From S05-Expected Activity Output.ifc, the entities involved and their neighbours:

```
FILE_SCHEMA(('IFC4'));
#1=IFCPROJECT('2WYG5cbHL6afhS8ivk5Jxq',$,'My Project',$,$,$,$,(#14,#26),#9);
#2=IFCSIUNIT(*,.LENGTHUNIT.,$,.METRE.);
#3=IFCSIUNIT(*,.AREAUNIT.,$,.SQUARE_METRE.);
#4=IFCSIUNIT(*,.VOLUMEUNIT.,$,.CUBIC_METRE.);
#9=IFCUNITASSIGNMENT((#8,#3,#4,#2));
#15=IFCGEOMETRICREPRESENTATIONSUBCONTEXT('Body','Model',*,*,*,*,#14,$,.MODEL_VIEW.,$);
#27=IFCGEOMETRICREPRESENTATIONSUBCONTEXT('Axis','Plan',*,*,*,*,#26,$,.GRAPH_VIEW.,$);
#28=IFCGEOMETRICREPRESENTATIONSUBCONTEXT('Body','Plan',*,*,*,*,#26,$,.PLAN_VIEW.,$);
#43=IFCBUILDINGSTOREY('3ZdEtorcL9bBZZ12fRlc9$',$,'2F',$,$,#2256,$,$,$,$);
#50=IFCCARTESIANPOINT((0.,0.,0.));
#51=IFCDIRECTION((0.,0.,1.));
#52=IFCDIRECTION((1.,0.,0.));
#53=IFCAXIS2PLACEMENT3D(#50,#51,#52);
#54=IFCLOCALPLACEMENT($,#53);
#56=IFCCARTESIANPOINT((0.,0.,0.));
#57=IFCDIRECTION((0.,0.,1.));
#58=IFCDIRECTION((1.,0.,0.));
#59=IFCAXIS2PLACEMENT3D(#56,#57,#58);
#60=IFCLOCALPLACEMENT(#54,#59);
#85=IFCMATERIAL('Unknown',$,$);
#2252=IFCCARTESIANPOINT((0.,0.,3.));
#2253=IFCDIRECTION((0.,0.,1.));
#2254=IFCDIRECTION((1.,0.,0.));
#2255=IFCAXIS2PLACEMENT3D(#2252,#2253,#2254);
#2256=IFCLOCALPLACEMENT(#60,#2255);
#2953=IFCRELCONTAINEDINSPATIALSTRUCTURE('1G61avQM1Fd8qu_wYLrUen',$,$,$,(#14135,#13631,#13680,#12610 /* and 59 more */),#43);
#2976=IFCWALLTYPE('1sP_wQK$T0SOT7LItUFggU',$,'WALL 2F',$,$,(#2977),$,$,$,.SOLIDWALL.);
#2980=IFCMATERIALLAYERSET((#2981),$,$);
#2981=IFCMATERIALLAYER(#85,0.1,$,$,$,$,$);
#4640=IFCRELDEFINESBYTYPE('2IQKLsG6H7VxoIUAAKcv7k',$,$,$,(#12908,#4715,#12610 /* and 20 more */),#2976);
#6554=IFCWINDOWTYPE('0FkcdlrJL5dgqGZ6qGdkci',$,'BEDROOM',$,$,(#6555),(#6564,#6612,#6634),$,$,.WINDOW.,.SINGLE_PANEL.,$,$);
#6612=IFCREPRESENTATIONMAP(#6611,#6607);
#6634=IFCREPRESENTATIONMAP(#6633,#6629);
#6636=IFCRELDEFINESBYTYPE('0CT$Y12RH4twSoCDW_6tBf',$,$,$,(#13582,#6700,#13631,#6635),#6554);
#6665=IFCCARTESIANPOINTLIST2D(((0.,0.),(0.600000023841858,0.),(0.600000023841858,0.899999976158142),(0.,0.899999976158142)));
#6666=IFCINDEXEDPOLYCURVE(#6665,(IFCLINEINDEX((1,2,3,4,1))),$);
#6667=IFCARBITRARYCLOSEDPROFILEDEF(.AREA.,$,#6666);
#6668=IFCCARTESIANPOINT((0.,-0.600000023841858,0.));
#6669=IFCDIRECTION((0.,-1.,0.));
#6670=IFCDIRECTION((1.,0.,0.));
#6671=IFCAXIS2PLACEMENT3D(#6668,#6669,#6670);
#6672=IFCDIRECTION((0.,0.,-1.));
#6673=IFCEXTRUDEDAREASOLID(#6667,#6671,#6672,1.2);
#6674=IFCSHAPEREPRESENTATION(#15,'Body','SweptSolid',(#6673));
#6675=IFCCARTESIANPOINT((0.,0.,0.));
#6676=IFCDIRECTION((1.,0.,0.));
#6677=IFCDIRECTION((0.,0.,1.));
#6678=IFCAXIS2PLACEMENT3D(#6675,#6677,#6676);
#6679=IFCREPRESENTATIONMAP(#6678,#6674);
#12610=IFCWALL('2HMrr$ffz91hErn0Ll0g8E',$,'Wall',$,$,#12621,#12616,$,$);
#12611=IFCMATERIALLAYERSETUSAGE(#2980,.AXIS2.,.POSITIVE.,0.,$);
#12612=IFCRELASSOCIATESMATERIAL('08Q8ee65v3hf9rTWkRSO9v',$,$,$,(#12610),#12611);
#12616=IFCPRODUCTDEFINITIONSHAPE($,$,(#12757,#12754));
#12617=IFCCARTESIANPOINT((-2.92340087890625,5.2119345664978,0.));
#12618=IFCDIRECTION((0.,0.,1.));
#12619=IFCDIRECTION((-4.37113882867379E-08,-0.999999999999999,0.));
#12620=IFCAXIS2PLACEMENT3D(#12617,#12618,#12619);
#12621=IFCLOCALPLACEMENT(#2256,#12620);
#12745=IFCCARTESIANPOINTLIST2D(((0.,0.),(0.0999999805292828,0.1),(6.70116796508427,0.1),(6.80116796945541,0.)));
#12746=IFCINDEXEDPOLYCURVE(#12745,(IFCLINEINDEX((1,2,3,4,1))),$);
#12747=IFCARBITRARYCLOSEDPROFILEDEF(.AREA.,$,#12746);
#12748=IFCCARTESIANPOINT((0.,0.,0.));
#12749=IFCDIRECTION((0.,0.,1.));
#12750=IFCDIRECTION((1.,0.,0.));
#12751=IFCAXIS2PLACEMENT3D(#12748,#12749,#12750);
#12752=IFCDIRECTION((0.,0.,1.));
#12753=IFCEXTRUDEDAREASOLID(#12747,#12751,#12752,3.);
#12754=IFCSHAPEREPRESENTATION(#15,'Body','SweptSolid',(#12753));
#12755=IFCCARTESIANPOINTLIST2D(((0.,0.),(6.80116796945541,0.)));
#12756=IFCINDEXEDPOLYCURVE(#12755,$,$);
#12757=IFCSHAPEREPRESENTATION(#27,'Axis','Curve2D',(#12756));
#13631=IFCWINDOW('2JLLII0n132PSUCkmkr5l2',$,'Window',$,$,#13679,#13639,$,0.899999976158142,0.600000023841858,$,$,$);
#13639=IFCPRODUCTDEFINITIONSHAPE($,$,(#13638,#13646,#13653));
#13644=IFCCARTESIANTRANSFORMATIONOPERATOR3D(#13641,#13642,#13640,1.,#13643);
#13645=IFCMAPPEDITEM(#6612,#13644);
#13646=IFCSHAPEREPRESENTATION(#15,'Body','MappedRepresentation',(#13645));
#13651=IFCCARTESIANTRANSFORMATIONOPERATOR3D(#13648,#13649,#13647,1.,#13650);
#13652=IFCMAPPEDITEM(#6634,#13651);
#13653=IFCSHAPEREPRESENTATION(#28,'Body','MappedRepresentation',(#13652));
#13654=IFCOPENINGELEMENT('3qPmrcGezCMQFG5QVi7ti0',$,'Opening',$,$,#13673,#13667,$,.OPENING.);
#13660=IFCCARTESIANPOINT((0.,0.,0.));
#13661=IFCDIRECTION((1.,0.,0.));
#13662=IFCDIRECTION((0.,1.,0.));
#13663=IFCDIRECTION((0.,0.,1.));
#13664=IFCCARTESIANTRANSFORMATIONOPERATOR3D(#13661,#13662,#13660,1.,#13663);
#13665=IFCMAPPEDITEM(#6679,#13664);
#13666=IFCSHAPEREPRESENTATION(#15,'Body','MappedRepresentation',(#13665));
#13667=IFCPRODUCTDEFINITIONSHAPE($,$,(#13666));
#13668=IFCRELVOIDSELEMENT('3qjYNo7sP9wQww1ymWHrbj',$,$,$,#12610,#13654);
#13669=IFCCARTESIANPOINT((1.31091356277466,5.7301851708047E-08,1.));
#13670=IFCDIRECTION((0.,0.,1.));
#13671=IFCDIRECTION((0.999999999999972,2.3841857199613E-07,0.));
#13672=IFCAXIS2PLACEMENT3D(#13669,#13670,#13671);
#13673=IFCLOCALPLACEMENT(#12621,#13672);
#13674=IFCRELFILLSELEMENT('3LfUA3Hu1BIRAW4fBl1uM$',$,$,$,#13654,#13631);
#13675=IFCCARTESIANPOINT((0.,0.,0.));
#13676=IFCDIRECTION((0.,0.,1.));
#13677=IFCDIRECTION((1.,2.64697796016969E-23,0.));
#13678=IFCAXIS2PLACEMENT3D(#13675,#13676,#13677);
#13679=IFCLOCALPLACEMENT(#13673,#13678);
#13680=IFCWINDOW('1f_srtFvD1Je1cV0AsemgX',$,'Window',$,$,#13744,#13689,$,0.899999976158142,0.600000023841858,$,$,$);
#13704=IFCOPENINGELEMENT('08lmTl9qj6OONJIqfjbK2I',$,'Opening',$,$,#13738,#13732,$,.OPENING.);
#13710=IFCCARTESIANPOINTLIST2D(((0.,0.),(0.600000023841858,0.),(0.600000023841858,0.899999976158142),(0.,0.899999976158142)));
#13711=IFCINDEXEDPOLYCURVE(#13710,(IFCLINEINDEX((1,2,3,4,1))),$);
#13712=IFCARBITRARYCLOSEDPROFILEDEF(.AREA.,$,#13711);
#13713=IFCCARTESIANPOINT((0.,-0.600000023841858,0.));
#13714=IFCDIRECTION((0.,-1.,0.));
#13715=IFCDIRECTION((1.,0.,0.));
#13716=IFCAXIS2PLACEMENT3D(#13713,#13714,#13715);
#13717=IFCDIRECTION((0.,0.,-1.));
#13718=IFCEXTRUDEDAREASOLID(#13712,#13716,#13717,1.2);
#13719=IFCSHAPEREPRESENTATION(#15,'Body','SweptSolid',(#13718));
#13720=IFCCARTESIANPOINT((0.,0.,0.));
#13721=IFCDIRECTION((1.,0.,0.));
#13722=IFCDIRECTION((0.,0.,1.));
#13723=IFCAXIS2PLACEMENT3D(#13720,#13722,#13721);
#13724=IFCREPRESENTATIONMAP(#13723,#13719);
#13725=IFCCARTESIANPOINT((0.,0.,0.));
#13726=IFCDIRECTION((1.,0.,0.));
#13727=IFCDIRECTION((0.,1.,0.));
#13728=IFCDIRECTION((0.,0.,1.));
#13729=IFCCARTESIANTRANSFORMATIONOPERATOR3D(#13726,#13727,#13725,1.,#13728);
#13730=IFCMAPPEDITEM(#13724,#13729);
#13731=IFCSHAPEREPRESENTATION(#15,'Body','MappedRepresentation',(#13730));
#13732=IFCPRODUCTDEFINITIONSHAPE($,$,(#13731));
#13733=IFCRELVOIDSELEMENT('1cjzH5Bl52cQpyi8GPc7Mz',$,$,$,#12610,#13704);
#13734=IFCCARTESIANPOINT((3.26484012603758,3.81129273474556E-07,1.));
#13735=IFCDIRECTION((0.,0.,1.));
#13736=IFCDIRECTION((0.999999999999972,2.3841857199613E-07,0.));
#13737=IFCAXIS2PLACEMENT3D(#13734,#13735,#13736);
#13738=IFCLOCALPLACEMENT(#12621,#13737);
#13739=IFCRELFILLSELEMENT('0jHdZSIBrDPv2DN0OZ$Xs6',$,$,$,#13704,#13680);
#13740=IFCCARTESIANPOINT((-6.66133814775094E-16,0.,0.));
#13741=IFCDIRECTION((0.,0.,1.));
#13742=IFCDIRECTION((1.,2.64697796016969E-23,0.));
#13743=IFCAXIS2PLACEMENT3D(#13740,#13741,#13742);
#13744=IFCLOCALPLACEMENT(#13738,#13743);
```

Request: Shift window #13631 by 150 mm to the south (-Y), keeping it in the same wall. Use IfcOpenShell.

```python
import ifcopenshell
import ifcopenshell.api.geometry
import ifcopenshell.util.placement
import ifcopenshell.util.unit

model = ifcopenshell.open("S05-Expected Activity Output.ifc")
unit_scale = ifcopenshell.util.unit.calculate_unit_scale(model)

window = model.by_guid("2JLLII0n132PSUCkmkr5l2")
opening = window.FillsVoids[0].RelatingOpeningElement
wall = opening.VoidsElements[0].RelatingBuildingElement

wall_matrix = ifcopenshell.util.placement.get_local_placement(wall.ObjectPlacement)
shift = wall_matrix[:3, 0] * 0.15 / unit_scale
before = ifcopenshell.util.placement.get_local_placement(window.ObjectPlacement)[:3, 3].copy()

# The window is placed relative to its opening, so it follows when the opening moves.
matrix = ifcopenshell.util.placement.get_local_placement(opening.ObjectPlacement)
matrix[:3, 3] += shift
ifcopenshell.api.geometry.edit_object_placement(
    model, product=opening, matrix=matrix, is_si=False, should_transform_children=True
)

after = ifcopenshell.util.placement.get_local_placement(window.ObjectPlacement)[:3, 3]
print("window moved by", (after - before).round(3) + 0.0)

model.write("S05-Expected Activity Output_v2.ifc")
```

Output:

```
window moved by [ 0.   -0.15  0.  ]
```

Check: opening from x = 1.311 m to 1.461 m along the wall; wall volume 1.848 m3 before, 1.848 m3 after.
